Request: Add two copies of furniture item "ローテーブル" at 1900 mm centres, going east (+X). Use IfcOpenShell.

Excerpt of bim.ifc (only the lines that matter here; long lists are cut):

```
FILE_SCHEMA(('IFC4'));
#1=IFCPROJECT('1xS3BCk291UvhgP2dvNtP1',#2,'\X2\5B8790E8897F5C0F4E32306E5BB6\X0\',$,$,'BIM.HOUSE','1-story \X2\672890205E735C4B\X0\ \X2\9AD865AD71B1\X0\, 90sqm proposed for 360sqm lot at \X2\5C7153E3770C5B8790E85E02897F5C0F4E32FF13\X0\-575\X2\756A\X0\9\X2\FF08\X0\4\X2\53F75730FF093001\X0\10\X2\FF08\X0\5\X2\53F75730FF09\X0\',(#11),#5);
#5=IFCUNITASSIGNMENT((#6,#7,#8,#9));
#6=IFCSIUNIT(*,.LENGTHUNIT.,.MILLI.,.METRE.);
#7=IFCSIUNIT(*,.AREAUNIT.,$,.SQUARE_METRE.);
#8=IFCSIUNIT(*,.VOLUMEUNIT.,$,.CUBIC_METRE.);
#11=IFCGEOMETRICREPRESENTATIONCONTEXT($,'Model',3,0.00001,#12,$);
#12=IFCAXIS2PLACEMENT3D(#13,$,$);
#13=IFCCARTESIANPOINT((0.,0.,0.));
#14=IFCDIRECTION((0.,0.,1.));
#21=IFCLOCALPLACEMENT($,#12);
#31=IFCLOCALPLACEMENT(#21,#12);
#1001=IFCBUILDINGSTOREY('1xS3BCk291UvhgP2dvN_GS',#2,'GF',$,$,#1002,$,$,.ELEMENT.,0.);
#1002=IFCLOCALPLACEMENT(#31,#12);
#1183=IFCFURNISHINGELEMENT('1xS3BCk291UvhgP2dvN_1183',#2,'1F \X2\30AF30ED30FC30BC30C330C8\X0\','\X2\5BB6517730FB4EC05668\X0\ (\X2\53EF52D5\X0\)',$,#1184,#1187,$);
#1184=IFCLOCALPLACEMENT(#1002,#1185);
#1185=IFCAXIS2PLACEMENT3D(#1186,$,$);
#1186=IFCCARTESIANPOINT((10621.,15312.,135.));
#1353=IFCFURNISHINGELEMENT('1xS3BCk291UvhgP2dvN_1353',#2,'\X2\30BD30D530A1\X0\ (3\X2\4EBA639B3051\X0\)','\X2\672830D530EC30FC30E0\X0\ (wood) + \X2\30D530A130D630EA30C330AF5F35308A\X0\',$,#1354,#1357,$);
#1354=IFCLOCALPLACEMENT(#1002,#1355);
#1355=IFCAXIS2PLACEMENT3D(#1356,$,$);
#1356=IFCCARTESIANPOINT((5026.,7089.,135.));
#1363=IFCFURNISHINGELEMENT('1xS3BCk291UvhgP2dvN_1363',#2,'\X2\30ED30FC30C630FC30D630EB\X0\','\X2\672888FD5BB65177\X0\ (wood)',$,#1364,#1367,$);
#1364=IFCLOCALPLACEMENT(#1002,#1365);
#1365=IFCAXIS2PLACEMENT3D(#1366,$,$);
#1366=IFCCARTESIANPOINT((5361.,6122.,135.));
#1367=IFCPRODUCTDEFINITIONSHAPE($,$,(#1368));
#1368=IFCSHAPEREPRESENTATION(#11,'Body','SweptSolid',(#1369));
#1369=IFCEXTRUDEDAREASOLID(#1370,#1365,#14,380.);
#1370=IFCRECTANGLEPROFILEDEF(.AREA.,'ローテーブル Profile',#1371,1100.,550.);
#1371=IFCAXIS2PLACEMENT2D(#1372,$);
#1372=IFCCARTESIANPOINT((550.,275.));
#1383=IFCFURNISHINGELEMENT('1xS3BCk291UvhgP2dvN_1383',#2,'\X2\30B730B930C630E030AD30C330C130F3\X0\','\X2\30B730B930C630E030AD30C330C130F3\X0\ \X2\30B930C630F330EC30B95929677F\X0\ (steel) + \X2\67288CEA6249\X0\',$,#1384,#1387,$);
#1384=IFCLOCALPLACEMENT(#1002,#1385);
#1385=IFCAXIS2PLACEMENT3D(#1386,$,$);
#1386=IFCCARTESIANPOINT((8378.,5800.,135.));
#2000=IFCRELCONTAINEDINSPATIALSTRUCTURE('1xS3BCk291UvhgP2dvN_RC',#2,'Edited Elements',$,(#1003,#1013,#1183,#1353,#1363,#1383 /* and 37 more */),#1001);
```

```python
import numpy as np
import ifcopenshell
import ifcopenshell.api.geometry
import ifcopenshell.api.root
import ifcopenshell.util.element
import ifcopenshell.util.placement
import ifcopenshell.util.unit

model = ifcopenshell.open("bim.ifc")
unit_scale = ifcopenshell.util.unit.calculate_unit_scale(model)


def reuse_history(source, copy):
    """copy_class also copies each property set's owner history, people and application; keep the originals."""
    for rel in copy.IsDefinedBy:
        if rel.is_a("IfcRelDefinesByProperties") and (history := rel.RelatingPropertyDefinition.OwnerHistory):
            rel.RelatingPropertyDefinition.OwnerHistory = source.OwnerHistory
            ifcopenshell.util.element.remove_deep2(model, history)


source = model.by_guid("1xS3BCk291UvhgP2dvN_1363")
base = ifcopenshell.util.placement.get_local_placement(source.ObjectPlacement)
step = np.array([1.0, 0.0, 0.0]) * 1.9 / unit_scale

for i in range(1, 3):
    copy = ifcopenshell.api.root.copy_class(model, product=source)
    copy.Representation = ifcopenshell.util.element.copy_deep(
        model, source.Representation, exclude=["IfcGeometricRepresentationContext", "IfcRepresentationMap"]
    )
    reuse_history(source, copy)
    matrix = base.copy()
    matrix[:3, 3] += i * step
    print("added at", matrix[:3, 3].round(3) + 0.0)
    ifcopenshell.api.geometry.edit_object_placement(model, product=copy, matrix=matrix, is_si=False)

model.write("bim-out.ifc")
```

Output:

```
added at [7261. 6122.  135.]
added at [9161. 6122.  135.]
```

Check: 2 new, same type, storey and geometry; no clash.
